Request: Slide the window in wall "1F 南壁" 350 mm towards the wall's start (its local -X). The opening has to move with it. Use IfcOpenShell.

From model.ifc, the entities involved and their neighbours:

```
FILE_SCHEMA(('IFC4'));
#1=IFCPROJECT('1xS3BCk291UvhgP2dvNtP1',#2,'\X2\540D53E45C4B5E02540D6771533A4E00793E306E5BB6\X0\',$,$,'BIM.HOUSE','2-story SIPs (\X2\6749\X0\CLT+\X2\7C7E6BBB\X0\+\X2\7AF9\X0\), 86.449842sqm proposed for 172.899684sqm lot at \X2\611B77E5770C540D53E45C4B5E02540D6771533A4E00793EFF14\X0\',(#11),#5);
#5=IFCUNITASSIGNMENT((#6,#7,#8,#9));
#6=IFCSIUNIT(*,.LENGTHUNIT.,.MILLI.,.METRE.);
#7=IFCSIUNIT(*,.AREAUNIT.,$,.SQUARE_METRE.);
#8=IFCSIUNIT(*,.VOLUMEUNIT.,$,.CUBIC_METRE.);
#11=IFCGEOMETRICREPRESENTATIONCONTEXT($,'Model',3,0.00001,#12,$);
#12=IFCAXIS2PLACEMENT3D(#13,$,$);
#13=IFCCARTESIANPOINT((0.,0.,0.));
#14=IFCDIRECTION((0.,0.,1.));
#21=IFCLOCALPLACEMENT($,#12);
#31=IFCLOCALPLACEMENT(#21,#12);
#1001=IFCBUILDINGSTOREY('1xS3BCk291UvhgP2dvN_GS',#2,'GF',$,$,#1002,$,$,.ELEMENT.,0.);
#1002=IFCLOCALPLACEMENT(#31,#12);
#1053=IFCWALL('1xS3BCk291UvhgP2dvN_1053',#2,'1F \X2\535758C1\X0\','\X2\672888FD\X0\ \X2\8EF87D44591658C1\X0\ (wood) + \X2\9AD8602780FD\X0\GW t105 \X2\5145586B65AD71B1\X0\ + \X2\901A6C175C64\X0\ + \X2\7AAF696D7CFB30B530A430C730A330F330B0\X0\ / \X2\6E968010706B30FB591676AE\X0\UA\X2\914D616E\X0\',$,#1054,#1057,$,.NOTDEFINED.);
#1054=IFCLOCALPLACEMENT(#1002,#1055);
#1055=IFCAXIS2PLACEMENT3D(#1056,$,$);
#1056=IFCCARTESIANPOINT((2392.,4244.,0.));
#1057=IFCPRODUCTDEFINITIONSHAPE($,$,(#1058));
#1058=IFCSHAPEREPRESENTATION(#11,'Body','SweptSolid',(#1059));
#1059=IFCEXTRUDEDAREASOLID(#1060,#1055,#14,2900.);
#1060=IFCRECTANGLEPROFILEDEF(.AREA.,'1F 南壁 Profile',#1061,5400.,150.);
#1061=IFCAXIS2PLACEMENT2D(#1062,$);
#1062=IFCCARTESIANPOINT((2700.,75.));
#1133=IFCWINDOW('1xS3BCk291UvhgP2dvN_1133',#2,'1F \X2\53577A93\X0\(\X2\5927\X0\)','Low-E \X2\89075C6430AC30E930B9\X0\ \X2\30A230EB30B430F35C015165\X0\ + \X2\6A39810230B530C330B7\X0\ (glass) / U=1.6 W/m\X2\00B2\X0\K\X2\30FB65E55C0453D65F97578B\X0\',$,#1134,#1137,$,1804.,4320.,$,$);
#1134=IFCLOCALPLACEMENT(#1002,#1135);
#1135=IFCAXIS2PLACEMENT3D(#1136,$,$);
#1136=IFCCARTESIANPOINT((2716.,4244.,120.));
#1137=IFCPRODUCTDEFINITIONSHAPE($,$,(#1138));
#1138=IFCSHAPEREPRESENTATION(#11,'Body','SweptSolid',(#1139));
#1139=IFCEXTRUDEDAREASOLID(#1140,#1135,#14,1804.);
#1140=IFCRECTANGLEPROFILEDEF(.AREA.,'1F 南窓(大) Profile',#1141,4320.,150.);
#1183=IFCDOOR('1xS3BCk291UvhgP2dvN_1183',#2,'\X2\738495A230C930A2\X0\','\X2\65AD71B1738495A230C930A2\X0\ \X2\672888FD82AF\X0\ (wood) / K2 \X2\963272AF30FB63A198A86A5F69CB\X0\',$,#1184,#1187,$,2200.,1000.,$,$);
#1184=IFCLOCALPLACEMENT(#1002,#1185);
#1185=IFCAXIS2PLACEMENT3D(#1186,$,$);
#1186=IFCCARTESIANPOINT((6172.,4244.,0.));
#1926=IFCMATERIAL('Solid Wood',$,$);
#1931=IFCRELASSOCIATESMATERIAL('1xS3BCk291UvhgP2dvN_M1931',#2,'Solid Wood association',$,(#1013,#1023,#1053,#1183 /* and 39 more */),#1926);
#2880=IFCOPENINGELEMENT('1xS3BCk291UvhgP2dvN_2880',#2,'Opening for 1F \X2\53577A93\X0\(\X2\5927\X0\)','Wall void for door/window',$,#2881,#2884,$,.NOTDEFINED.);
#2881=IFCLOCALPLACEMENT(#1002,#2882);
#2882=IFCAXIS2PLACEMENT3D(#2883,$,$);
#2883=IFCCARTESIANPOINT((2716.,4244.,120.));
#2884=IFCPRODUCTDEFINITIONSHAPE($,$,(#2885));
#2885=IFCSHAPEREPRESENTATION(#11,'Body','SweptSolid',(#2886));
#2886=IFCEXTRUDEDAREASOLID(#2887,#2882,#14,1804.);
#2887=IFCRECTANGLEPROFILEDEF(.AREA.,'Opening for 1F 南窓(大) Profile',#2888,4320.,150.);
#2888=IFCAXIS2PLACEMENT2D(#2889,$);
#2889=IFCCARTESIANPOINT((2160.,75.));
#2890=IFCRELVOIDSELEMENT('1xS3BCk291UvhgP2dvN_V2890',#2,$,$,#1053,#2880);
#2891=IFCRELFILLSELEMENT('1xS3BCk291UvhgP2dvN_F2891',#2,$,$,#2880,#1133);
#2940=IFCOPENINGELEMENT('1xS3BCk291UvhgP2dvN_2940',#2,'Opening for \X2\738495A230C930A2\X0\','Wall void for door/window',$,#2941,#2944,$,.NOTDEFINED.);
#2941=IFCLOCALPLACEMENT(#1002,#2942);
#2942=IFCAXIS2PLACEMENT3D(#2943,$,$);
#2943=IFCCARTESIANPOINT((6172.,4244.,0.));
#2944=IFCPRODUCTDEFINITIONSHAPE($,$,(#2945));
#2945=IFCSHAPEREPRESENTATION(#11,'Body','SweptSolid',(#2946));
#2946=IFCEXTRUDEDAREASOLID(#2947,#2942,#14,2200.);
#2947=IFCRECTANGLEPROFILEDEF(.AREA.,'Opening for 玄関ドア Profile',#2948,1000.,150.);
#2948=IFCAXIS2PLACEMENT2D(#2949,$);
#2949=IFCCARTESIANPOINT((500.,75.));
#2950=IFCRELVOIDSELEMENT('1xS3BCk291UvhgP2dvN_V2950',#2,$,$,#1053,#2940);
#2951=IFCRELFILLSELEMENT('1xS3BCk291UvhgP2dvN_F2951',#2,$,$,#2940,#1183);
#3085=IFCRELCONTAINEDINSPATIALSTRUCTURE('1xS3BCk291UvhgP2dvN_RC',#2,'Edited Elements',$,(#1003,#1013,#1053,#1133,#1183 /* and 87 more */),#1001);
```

```python
import ifcopenshell
import ifcopenshell.api.geometry
import ifcopenshell.util.placement
import ifcopenshell.util.unit

model = ifcopenshell.open("model.ifc")
unit_scale = ifcopenshell.util.unit.calculate_unit_scale(model)

window = model.by_guid("1xS3BCk291UvhgP2dvN_1133")
opening = window.FillsVoids[0].RelatingOpeningElement
wall = opening.VoidsElements[0].RelatingBuildingElement

wall_matrix = ifcopenshell.util.placement.get_local_placement(wall.ObjectPlacement)
shift = wall_matrix[:3, 0] * -0.35 / unit_scale
before = ifcopenshell.util.placement.get_local_placement(window.ObjectPlacement)[:3, 3].copy()

# The window is not placed relative to its opening, so move both.
for product in (opening, window):
    matrix = ifcopenshell.util.placement.get_local_placement(product.ObjectPlacement)
    matrix[:3, 3] += shift
    ifcopenshell.api.geometry.edit_object_placement(model, product=product, matrix=matrix, is_si=False)

after = ifcopenshell.util.placement.get_local_placement(window.ObjectPlacement)[:3, 3]
print("window moved by", (after - before).round(3) + 0.0)

model.write("model_edited.ifc")
```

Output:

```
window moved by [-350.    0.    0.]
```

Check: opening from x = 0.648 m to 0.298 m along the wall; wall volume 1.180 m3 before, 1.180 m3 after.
